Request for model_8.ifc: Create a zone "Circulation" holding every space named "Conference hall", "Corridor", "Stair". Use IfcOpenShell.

First a look at what the model holds.

```python
import ifcopenshell

model = ifcopenshell.open("model_8.ifc")
print(model.schema)
seen = {}
for space in model.by_type("IfcSpace"):
    seen[space.LongName] = seen.get(space.LongName, 0) + 1
for name, count in sorted(seen.items(), key=str):
    print(count, "x", name)
print("zones:", [z.Name for z in model.by_type("IfcZone")][:20])
```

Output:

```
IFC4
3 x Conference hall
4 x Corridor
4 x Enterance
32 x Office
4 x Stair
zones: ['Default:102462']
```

```python
import ifcopenshell
import ifcopenshell.api.group
import ifcopenshell.api.root

model = ifcopenshell.open("model_8.ifc")

names = {"Conference hall", "Corridor", "Stair"}
spaces = [s for s in model.by_type("IfcSpace") if s.LongName in names]

zone = ifcopenshell.api.root.create_entity(model, ifc_class="IfcZone", name="Circulation")
ifcopenshell.api.group.assign_group(model, products=spaces, group=zone)
print(len(spaces), "spaces in", zone.Name)

model.write("model_8_updated.ifc")
```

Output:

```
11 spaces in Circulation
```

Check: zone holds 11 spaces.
